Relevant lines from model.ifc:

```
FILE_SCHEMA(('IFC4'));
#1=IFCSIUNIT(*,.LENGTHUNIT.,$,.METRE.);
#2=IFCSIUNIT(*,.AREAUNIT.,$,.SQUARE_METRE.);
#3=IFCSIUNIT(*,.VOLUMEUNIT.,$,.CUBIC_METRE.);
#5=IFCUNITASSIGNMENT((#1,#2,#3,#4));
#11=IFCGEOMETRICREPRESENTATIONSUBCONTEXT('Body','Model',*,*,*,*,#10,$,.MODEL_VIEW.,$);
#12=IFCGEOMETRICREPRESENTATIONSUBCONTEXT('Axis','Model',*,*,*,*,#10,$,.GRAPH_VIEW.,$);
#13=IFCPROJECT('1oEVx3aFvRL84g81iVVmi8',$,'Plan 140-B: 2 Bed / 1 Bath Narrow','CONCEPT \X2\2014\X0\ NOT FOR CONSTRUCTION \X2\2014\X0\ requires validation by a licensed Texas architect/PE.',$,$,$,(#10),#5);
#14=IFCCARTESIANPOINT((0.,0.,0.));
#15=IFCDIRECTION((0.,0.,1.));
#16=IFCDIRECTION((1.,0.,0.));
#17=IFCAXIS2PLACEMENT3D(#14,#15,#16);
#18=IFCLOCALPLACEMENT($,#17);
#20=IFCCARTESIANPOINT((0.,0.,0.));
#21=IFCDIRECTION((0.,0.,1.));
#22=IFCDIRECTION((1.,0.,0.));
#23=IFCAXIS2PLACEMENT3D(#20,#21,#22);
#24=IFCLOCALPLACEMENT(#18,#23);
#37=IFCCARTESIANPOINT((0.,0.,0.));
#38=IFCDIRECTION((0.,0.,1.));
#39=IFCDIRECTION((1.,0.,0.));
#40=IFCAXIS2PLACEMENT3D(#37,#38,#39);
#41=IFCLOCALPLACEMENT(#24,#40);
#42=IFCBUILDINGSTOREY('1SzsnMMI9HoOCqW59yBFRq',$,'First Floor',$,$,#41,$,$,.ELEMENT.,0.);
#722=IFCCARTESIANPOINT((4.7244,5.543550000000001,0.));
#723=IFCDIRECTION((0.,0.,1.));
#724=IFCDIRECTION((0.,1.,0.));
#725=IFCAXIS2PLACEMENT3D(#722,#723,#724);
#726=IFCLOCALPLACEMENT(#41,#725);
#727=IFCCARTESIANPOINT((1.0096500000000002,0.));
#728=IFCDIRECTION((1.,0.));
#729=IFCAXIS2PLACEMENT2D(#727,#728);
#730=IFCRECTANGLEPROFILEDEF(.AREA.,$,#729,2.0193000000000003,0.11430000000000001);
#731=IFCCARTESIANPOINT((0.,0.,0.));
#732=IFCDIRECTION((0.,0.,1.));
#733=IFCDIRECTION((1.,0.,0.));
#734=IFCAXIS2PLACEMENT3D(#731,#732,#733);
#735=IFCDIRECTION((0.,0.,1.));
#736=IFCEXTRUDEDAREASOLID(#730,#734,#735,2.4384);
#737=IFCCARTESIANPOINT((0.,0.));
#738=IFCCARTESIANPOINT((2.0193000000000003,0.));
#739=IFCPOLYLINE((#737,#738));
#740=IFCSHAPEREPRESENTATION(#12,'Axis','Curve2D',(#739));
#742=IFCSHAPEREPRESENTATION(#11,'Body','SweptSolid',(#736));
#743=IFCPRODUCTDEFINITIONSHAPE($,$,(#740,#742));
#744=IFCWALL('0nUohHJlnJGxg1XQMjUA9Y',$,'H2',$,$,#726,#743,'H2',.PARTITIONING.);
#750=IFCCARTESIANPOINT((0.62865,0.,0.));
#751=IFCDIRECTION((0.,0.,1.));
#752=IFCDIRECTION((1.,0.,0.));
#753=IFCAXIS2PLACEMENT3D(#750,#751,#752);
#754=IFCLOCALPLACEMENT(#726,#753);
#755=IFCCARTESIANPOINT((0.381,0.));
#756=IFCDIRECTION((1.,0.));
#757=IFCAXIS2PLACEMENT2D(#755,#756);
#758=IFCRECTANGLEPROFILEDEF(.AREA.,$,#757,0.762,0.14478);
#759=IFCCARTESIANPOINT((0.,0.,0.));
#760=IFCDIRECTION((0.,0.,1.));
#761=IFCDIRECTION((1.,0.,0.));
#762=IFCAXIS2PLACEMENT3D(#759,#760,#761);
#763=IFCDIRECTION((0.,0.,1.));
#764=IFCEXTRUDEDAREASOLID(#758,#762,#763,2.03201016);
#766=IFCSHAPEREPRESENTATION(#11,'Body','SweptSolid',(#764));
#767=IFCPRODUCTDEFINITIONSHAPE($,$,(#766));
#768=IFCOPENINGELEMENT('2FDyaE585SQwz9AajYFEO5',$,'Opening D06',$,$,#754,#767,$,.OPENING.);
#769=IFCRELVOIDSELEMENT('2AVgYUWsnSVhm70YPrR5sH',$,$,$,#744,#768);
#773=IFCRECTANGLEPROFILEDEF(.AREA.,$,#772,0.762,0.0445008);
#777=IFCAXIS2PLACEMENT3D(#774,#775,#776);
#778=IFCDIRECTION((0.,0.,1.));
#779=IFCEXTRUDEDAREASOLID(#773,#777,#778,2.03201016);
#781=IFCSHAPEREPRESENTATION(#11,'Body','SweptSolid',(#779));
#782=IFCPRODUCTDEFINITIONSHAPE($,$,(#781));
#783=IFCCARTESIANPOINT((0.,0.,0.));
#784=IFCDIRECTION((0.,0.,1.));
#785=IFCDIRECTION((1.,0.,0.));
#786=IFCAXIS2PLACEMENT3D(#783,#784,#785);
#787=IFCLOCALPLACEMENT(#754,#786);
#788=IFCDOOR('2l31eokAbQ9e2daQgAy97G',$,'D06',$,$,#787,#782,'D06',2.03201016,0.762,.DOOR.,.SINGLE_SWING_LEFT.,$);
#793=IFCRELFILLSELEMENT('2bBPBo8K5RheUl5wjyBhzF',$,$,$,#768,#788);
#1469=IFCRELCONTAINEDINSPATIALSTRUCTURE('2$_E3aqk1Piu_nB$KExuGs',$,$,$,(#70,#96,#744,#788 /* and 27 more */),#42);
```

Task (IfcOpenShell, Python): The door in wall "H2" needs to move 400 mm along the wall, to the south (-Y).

```python
import ifcopenshell
import ifcopenshell.api.geometry
import ifcopenshell.util.placement
import ifcopenshell.util.unit

model = ifcopenshell.open("model.ifc")
unit_scale = ifcopenshell.util.unit.calculate_unit_scale(model)

door = model.by_id(788)
opening = door.FillsVoids[0].RelatingOpeningElement
wall = opening.VoidsElements[0].RelatingBuildingElement

wall_matrix = ifcopenshell.util.placement.get_local_placement(wall.ObjectPlacement)
shift = wall_matrix[:3, 0] * -0.4 / unit_scale
before = ifcopenshell.util.placement.get_local_placement(door.ObjectPlacement)[:3, 3].copy()

# The door is placed relative to its opening, so it follows when the opening moves.
matrix = ifcopenshell.util.placement.get_local_placement(opening.ObjectPlacement)
matrix[:3, 3] += shift
ifcopenshell.api.geometry.edit_object_placement(
    model, product=opening, matrix=matrix, is_si=False, should_transform_children=True
)

after = ifcopenshell.util.placement.get_local_placement(door.ObjectPlacement)[:3, 3]
print("door moved by", (after - before).round(3) + 0.0)

model.write("model_rev.ifc")
```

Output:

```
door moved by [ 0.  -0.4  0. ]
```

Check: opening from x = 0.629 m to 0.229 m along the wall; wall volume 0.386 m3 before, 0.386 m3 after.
